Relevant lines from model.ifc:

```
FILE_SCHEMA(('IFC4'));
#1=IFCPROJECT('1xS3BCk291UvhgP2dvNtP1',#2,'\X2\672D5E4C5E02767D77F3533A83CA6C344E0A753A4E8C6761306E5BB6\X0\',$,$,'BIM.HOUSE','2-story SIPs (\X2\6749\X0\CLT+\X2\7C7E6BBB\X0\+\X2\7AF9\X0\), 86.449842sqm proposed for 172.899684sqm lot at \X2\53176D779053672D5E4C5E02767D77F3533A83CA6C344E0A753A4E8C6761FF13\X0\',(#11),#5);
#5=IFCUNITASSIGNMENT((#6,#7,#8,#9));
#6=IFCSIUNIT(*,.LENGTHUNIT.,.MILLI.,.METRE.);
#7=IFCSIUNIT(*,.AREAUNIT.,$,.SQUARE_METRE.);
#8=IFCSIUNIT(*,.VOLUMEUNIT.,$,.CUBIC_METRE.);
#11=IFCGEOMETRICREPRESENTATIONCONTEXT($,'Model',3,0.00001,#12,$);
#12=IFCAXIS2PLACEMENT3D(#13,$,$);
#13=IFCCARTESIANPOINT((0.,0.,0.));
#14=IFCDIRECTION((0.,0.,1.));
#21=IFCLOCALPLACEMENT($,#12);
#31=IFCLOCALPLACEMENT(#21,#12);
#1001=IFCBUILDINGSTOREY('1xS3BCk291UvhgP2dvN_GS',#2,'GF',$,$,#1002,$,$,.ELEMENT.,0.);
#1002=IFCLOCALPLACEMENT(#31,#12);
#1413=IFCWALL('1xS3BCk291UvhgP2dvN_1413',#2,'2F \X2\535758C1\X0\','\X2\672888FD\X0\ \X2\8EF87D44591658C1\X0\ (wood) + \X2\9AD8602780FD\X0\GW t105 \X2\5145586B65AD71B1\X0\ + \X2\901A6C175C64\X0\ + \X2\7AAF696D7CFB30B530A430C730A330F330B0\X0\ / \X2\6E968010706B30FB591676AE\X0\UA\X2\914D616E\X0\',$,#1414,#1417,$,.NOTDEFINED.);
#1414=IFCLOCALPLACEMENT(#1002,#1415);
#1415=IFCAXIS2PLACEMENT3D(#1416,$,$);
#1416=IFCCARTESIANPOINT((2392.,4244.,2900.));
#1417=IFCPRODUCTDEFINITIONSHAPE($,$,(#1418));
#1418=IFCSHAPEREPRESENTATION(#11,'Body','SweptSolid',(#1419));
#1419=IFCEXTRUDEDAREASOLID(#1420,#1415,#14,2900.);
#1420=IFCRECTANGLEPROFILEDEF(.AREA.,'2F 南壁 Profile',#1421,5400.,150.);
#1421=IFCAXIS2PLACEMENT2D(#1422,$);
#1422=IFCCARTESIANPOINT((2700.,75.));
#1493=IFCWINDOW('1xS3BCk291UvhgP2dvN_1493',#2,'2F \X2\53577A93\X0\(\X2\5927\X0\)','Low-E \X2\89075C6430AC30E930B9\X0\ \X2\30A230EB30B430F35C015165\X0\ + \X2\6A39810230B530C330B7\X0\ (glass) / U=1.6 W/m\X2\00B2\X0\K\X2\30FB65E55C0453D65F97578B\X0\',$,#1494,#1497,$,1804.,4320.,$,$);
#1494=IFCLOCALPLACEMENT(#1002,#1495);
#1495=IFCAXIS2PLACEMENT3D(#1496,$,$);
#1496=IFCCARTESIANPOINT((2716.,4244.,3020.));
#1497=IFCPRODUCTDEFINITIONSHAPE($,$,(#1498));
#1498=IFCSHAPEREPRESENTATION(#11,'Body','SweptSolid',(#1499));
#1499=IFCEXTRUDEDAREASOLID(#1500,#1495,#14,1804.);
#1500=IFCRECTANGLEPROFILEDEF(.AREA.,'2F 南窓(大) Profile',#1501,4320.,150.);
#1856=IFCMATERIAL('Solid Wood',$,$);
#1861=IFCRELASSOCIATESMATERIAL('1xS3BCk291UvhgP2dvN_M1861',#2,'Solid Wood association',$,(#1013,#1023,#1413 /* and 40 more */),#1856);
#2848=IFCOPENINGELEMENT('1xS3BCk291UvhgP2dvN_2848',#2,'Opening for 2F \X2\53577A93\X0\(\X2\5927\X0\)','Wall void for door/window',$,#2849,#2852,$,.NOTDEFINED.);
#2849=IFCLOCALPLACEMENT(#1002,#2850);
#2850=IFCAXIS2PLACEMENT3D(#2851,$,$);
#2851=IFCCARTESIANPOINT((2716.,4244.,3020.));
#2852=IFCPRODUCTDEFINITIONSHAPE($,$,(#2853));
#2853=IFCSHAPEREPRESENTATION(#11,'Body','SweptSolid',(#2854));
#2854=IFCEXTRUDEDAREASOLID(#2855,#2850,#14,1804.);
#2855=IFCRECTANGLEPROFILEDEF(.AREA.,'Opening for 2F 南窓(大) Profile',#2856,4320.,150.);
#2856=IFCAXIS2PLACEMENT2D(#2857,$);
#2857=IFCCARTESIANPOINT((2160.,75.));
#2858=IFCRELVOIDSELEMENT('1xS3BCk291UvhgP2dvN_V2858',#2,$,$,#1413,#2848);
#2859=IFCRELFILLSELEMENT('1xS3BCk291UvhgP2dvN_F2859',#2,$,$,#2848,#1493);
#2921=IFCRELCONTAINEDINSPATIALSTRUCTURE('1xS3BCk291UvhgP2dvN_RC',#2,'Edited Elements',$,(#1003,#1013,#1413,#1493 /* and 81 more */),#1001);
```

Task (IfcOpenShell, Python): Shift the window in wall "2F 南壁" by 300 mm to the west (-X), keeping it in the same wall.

```python
import ifcopenshell
import ifcopenshell.api.geometry
import ifcopenshell.util.placement
import ifcopenshell.util.unit

model = ifcopenshell.open("model.ifc")
unit_scale = ifcopenshell.util.unit.calculate_unit_scale(model)

window = model.by_guid("1xS3BCk291UvhgP2dvN_1493")
opening = window.FillsVoids[0].RelatingOpeningElement
wall = opening.VoidsElements[0].RelatingBuildingElement

wall_matrix = ifcopenshell.util.placement.get_local_placement(wall.ObjectPlacement)
shift = wall_matrix[:3, 0] * -0.3 / unit_scale
before = ifcopenshell.util.placement.get_local_placement(window.ObjectPlacement)[:3, 3].copy()

# The window is not placed relative to its opening, so move both.
for product in (opening, window):
    matrix = ifcopenshell.util.placement.get_local_placement(product.ObjectPlacement)
    matrix[:3, 3] += shift
    ifcopenshell.api.geometry.edit_object_placement(model, product=product, matrix=matrix, is_si=False)

after = ifcopenshell.util.placement.get_local_placement(window.ObjectPlacement)[:3, 3]
print("window moved by", (after - before).round(3) + 0.0)

model.write("model-out.ifc")
```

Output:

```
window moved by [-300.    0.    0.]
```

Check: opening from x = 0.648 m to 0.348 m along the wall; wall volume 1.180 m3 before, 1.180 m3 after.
